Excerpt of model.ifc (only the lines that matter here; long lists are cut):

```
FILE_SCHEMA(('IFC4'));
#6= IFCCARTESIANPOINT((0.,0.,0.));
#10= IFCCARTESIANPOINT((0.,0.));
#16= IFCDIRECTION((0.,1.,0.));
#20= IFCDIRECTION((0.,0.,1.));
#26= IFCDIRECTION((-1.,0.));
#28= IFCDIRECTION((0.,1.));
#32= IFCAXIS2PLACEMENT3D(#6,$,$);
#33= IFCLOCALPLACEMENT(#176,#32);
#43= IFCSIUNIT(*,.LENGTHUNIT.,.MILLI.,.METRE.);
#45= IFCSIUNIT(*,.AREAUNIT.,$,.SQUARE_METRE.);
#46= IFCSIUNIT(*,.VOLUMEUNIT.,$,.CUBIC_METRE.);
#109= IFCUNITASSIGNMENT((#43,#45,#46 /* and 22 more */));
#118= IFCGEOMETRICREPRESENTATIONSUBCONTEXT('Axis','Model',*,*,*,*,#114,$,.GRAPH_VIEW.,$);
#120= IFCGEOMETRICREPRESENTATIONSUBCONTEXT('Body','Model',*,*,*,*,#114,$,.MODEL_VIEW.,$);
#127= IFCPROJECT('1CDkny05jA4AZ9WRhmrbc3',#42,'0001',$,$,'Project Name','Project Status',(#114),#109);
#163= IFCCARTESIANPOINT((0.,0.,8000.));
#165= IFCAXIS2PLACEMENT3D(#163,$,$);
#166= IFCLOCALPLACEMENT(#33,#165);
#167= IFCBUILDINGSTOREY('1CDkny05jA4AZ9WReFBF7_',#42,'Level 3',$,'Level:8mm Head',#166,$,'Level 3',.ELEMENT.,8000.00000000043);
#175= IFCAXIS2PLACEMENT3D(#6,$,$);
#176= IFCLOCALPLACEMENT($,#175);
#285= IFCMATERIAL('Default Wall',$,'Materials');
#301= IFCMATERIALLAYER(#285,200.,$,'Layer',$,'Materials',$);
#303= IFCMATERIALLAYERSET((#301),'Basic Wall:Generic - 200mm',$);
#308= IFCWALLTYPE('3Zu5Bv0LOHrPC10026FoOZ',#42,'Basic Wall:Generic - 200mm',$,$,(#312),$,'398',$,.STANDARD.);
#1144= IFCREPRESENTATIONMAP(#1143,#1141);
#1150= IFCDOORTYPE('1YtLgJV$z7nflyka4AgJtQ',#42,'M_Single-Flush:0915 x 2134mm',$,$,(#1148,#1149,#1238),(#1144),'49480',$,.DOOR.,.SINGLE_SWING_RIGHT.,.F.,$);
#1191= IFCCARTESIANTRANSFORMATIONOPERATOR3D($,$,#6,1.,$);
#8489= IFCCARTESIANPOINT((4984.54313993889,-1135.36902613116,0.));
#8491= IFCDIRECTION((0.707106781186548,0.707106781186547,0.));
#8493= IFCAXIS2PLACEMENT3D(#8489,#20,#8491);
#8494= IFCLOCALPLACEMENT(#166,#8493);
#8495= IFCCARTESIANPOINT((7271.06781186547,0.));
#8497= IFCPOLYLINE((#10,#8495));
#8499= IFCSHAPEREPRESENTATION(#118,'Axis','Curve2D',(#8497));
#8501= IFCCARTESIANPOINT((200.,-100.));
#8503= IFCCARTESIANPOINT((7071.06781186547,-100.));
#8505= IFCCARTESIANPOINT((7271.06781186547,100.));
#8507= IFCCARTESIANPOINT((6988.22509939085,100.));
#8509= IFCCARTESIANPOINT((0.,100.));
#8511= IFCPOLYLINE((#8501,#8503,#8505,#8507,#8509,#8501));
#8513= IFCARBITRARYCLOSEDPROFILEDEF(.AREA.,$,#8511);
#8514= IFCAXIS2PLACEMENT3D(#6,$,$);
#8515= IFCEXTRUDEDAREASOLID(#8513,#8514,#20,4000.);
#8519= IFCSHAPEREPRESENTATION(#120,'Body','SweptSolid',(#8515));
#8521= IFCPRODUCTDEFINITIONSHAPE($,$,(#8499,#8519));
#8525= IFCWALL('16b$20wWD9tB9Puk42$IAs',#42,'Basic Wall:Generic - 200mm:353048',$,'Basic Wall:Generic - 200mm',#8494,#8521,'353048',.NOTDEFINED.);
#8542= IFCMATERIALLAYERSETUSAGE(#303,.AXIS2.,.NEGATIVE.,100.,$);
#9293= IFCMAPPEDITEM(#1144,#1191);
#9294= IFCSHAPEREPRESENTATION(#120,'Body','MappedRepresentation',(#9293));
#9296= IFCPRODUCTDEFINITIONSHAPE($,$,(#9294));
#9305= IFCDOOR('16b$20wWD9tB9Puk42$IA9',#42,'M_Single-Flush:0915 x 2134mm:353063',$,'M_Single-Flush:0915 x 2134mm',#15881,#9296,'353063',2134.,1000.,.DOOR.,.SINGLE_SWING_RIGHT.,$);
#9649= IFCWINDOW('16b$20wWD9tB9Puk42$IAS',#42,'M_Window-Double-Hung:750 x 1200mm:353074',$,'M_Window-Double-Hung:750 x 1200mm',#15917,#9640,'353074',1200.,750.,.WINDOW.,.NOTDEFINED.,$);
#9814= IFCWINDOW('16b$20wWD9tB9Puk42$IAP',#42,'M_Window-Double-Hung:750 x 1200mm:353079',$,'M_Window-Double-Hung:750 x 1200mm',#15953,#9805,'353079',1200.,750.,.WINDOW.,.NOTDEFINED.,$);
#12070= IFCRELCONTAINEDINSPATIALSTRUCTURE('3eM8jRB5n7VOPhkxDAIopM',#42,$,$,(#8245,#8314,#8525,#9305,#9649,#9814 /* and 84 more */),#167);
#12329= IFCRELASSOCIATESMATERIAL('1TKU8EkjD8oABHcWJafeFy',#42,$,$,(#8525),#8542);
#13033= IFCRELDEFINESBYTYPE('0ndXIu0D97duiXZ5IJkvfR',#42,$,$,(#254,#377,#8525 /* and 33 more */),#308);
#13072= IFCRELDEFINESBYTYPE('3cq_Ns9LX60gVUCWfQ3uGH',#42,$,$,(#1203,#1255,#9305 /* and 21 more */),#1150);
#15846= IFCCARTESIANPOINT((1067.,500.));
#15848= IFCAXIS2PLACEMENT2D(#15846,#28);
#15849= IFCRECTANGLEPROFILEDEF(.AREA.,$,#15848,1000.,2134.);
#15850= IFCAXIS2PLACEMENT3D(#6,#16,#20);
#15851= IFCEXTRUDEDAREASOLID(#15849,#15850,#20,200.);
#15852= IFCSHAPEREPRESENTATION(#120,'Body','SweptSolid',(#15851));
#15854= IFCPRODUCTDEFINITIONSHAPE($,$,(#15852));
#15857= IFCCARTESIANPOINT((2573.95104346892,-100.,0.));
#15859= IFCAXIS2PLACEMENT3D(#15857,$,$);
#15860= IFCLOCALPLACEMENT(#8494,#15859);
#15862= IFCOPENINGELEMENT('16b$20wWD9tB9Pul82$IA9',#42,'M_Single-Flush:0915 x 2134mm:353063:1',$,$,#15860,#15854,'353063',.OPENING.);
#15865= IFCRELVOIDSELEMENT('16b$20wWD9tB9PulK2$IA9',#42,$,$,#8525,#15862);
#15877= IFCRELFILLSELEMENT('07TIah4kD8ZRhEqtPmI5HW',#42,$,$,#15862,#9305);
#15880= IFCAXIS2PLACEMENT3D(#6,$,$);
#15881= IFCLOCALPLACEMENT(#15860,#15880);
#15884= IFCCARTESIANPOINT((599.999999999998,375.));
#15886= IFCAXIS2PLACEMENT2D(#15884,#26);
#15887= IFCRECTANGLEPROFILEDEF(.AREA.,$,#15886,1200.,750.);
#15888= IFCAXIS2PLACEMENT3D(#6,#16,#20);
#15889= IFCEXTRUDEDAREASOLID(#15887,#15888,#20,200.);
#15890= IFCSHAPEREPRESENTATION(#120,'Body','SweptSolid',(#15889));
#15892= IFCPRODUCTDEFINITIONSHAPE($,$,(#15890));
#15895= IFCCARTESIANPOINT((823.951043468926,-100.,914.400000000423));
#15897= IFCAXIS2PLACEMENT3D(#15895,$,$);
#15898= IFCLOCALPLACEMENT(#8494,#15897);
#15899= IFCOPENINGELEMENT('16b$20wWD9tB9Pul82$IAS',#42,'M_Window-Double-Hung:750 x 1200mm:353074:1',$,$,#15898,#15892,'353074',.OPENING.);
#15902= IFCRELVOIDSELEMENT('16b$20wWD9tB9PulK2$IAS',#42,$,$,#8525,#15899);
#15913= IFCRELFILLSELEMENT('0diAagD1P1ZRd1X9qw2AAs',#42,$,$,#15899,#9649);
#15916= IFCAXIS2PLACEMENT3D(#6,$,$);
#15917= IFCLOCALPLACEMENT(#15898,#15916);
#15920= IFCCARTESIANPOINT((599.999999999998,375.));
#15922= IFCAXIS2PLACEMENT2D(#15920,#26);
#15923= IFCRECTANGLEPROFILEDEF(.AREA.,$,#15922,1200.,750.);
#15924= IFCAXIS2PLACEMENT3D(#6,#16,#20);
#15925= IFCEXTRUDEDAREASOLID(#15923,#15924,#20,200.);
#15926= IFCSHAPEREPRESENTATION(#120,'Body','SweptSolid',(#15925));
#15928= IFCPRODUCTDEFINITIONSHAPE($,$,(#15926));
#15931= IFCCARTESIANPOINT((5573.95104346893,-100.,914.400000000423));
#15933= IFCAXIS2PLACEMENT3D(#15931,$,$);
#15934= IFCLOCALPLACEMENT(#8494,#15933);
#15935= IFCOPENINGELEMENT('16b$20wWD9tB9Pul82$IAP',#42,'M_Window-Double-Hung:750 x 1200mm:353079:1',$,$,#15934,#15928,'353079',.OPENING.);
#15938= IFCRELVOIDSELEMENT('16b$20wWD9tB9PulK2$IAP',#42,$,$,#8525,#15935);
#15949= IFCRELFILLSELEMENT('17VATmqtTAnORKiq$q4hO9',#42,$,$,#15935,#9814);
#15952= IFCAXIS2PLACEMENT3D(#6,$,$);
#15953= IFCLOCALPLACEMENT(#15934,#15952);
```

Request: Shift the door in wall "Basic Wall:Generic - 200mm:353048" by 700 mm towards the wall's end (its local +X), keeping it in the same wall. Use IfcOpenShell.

```python
import ifcopenshell
import ifcopenshell.api.geometry
import ifcopenshell.util.placement
import ifcopenshell.util.unit

model = ifcopenshell.open("model.ifc")
unit_scale = ifcopenshell.util.unit.calculate_unit_scale(model)

door = model.by_guid("16b$20wWD9tB9Puk42$IA9")
opening = door.FillsVoids[0].RelatingOpeningElement
wall = opening.VoidsElements[0].RelatingBuildingElement

wall_matrix = ifcopenshell.util.placement.get_local_placement(wall.ObjectPlacement)
shift = wall_matrix[:3, 0] * 0.7 / unit_scale
before = ifcopenshell.util.placement.get_local_placement(door.ObjectPlacement)[:3, 3].copy()

# The door is placed relative to its opening, so it follows when the opening moves.
matrix = ifcopenshell.util.placement.get_local_placement(opening.ObjectPlacement)
matrix[:3, 3] += shift
ifcopenshell.api.geometry.edit_object_placement(
    model, product=opening, matrix=matrix, is_si=False, should_transform_children=True
)

after = ifcopenshell.util.placement.get_local_placement(door.ObjectPlacement)[:3, 3]
print("door moved by", (after - before).round(3) + 0.0)

model.write("model-out.ifc")
```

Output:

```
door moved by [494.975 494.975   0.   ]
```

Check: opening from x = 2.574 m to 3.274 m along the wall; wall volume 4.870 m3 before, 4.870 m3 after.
